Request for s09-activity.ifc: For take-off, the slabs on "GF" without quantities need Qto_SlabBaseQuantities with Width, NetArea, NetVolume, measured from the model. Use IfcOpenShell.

First a look at what the model holds.

```python
import ifcopenshell
import ifcopenshell.util.element
import ifcopenshell.util.unit

model = ifcopenshell.open("s09-activity.ifc")
print(model.schema)
for unit_type in ("LENGTHUNIT", "AREAUNIT", "VOLUMEUNIT"):
    print(unit_type, ifcopenshell.util.unit.calculate_unit_scale(model, unit_type))
storey = next(s for s in model.by_type("IfcBuildingStorey") if s.Name == "GF")
slabs = [e for e in ifcopenshell.util.element.get_decomposition(storey) if e.is_a("IfcSlab")]
for e in sorted(slabs, key=lambda e: e.id()):
    print(e.id(), e.is_a(), e.Name, list(ifcopenshell.util.element.get_psets(e, qtos_only=True)), sep=" | ")
```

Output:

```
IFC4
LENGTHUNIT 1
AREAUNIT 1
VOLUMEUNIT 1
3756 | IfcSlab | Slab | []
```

```python
import ifcopenshell
import ifcopenshell.api.pset
import ifcopenshell.geom
import ifcopenshell.util.element
import ifcopenshell.util.shape
import ifcopenshell.util.unit

model = ifcopenshell.open("s09-activity.ifc")
unit_scale = ifcopenshell.util.unit.calculate_unit_scale(model)
area_scale = ifcopenshell.util.unit.calculate_unit_scale(model, "AREAUNIT")
volume_scale = ifcopenshell.util.unit.calculate_unit_scale(model, "VOLUMEUNIT")
settings = ifcopenshell.geom.settings()

storey = next(s for s in model.by_type("IfcBuildingStorey") if s.Name == "GF")
slabs = [e for e in ifcopenshell.util.element.get_decomposition(storey) if e.is_a("IfcSlab")]

for e in sorted(slabs, key=lambda e: e.id()):
    if ifcopenshell.util.element.get_psets(e, qtos_only=True, should_inherit=False):
        continue
    # Geometry comes back in metres, in the element's own axes.
    shape = ifcopenshell.geom.create_shape(settings, e)
    values = {
        "Width": ifcopenshell.util.shape.get_z(shape.geometry) / unit_scale,
        "NetArea": ifcopenshell.util.shape.get_footprint_area(shape.geometry) / area_scale,
        "NetVolume": ifcopenshell.util.shape.get_volume(shape.geometry) / volume_scale,
    }
    qto = ifcopenshell.api.pset.add_qto(model, product=e, name="Qto_SlabBaseQuantities")
    ifcopenshell.api.pset.edit_qto(model, qto=qto, properties=values)
    print(e.id(), {k: round(v, 3) for k, v in values.items()})

model.write("s09-activity_updated.ifc")
```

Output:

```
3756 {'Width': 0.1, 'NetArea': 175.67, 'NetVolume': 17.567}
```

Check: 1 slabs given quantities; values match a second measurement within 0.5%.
